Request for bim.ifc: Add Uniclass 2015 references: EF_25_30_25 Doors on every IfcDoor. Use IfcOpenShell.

First a look at what the model holds.

```python
import ifcopenshell

model = ifcopenshell.open("bim.ifc")
print(model.schema)
print("classifications:", [c.Name for c in model.by_type("IfcClassification")])
for ifc_class in ("IfcDoor", "IfcRoof", "IfcStair", "IfcWall", "IfcWindow"):
    print(ifc_class, len(model.by_type(ifc_class)))
```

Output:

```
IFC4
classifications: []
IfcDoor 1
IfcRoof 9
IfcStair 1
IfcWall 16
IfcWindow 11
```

```python
import ifcopenshell
import ifcopenshell.api.classification

model = ifcopenshell.open("bim.ifc")

system = ifcopenshell.api.classification.add_classification(model, classification="Uniclass 2015")

codes = {
    "IfcDoor": ("EF_25_30_25", "Doors"),
}
for ifc_class, (code, name) in codes.items():
    products = model.by_type(ifc_class)
    ifcopenshell.api.classification.add_reference(
        model, products=products, classification=system, identification=code, name=name
    )
    print(code, len(products))

model.write("bim-out.ifc")
```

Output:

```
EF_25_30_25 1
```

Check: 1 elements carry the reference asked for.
